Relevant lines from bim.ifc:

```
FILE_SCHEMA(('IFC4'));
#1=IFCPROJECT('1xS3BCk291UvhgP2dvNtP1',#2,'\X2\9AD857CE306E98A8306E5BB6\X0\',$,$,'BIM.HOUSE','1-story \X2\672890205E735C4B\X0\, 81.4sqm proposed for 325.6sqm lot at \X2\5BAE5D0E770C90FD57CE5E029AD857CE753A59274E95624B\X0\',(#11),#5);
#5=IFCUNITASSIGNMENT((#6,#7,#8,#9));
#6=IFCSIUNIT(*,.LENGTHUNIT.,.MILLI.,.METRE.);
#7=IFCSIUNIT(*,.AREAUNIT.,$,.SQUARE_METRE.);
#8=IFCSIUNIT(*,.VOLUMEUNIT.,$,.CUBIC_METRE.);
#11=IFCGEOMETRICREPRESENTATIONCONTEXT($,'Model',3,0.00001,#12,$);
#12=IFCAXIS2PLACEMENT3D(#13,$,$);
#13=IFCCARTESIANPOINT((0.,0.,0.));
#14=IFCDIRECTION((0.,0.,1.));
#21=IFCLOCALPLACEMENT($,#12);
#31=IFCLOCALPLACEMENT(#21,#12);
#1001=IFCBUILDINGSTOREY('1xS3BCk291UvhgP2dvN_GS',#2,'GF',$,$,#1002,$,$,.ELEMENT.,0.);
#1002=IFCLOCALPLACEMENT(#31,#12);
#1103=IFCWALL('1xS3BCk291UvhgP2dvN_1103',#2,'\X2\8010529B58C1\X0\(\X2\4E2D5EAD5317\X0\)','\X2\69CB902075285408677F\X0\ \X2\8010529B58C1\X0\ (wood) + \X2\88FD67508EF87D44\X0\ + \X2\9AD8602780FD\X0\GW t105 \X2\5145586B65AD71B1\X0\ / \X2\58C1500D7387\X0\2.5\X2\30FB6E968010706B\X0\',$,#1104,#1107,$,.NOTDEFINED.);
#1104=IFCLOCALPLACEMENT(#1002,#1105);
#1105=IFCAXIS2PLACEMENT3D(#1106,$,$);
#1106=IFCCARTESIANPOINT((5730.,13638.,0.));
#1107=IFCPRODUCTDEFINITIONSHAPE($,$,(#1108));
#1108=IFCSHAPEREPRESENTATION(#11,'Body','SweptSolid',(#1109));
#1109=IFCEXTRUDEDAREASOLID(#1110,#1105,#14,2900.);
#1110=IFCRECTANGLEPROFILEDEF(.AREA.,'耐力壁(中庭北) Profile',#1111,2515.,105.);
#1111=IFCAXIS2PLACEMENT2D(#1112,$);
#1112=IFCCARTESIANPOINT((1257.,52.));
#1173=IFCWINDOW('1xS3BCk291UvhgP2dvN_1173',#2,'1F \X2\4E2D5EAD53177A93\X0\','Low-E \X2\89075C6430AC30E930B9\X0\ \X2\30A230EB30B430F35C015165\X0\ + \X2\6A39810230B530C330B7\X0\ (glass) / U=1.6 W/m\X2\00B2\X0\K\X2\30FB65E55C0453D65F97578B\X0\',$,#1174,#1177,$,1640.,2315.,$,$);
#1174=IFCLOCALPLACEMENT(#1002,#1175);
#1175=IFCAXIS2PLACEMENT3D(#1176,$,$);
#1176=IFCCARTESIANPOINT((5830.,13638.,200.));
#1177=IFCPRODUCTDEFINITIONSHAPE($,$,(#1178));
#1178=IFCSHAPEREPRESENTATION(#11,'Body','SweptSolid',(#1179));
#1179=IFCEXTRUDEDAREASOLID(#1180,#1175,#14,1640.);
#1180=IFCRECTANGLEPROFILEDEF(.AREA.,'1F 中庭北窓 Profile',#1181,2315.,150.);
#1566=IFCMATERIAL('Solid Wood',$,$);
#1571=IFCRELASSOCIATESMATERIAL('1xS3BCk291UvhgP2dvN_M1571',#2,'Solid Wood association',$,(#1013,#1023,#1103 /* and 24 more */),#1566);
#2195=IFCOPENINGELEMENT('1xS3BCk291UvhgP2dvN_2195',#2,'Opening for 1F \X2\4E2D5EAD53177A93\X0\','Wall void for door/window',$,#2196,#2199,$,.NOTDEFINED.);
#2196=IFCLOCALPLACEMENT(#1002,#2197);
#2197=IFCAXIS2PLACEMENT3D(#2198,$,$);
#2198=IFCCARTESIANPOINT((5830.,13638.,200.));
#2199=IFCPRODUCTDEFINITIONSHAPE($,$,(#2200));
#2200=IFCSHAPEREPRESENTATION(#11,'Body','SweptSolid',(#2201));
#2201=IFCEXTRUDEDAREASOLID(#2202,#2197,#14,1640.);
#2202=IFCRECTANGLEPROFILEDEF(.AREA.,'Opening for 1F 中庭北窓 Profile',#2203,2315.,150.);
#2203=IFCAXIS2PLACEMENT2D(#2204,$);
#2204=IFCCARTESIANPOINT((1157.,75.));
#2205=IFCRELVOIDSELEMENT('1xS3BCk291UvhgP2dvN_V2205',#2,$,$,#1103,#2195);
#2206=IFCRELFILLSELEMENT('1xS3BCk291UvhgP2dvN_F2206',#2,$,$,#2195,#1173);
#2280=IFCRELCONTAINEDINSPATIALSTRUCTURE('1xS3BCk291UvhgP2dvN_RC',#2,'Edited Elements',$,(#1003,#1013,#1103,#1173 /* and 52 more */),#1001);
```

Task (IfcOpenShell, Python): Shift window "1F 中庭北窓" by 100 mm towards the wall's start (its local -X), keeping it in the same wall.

```python
import ifcopenshell
import ifcopenshell.api.geometry
import ifcopenshell.util.placement
import ifcopenshell.util.unit

model = ifcopenshell.open("bim.ifc")
unit_scale = ifcopenshell.util.unit.calculate_unit_scale(model)

window = model.by_id(1173)
opening = window.FillsVoids[0].RelatingOpeningElement
wall = opening.VoidsElements[0].RelatingBuildingElement

wall_matrix = ifcopenshell.util.placement.get_local_placement(wall.ObjectPlacement)
shift = wall_matrix[:3, 0] * -0.1 / unit_scale
before = ifcopenshell.util.placement.get_local_placement(window.ObjectPlacement)[:3, 3].copy()

# The window is not placed relative to its opening, so move both.
for product in (opening, window):
    matrix = ifcopenshell.util.placement.get_local_placement(product.ObjectPlacement)
    matrix[:3, 3] += shift
    ifcopenshell.api.geometry.edit_object_placement(model, product=product, matrix=matrix, is_si=False)

after = ifcopenshell.util.placement.get_local_placement(window.ObjectPlacement)[:3, 3]
print("window moved by", (after - before).round(3) + 0.0)

model.write("bim_rev.ifc")
```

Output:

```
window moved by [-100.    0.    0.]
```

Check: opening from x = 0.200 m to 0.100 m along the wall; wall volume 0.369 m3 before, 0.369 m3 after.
